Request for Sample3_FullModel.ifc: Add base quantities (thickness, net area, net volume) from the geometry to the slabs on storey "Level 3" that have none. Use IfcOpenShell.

First a look at what the model holds.

```python
import ifcopenshell
import ifcopenshell.util.element
import ifcopenshell.util.unit

model = ifcopenshell.open("Sample3_FullModel.ifc")
print(model.schema)
for unit_type in ("LENGTHUNIT", "AREAUNIT", "VOLUMEUNIT"):
    print(unit_type, ifcopenshell.util.unit.calculate_unit_scale(model, unit_type))
storey = next(s for s in model.by_type("IfcBuildingStorey") if s.Name == "Level 3")
slabs = [e for e in ifcopenshell.util.element.get_decomposition(storey) if e.is_a("IfcSlab")]
for e in sorted(slabs, key=lambda e: e.id()):
    print(e.id(), e.is_a(), e.Name, list(ifcopenshell.util.element.get_psets(e, qtos_only=True)), sep=" | ")
```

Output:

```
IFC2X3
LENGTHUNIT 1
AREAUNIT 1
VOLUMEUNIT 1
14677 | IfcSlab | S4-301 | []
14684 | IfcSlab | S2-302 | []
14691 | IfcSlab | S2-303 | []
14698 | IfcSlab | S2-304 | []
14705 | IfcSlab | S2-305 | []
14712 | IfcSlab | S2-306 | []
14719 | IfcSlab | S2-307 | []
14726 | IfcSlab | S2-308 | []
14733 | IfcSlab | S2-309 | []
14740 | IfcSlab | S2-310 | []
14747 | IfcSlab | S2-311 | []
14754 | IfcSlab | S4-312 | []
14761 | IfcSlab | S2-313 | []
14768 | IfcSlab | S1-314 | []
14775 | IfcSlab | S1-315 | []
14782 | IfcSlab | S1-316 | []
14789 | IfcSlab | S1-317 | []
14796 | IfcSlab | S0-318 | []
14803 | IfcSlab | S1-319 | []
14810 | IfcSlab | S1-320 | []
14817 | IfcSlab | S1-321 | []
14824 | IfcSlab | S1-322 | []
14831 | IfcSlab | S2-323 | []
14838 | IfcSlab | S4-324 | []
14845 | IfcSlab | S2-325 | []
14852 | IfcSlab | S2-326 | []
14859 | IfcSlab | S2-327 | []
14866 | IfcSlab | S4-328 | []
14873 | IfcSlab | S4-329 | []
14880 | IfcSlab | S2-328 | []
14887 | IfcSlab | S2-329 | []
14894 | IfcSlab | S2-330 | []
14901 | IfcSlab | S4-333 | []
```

```python
import ifcopenshell
import ifcopenshell.api.pset
import ifcopenshell.geom
import ifcopenshell.util.element
import ifcopenshell.util.shape
import ifcopenshell.util.unit

model = ifcopenshell.open("Sample3_FullModel.ifc")
unit_scale = ifcopenshell.util.unit.calculate_unit_scale(model)
area_scale = ifcopenshell.util.unit.calculate_unit_scale(model, "AREAUNIT")
volume_scale = ifcopenshell.util.unit.calculate_unit_scale(model, "VOLUMEUNIT")
settings = ifcopenshell.geom.settings()

storey = next(s for s in model.by_type("IfcBuildingStorey") if s.Name == "Level 3")
slabs = [e for e in ifcopenshell.util.element.get_decomposition(storey) if e.is_a("IfcSlab")]

for e in sorted(slabs, key=lambda e: e.id()):
    if ifcopenshell.util.element.get_psets(e, qtos_only=True, should_inherit=False):
        continue
    # Geometry comes back in metres, in the element's own axes.
    shape = ifcopenshell.geom.create_shape(settings, e)
    values = {
        "Width": ifcopenshell.util.shape.get_z(shape.geometry) / unit_scale,
        "NetArea": ifcopenshell.util.shape.get_footprint_area(shape.geometry) / area_scale,
        "NetVolume": ifcopenshell.util.shape.get_volume(shape.geometry) / volume_scale,
    }
    qto = ifcopenshell.api.pset.add_qto(model, product=e, name="BaseQuantities")
    ifcopenshell.api.pset.edit_qto(model, qto=qto, properties=values)
    print(e.id(), {k: round(v, 3) for k, v in values.items()})

model.write("Sample3_FullModel_v2.ifc")
```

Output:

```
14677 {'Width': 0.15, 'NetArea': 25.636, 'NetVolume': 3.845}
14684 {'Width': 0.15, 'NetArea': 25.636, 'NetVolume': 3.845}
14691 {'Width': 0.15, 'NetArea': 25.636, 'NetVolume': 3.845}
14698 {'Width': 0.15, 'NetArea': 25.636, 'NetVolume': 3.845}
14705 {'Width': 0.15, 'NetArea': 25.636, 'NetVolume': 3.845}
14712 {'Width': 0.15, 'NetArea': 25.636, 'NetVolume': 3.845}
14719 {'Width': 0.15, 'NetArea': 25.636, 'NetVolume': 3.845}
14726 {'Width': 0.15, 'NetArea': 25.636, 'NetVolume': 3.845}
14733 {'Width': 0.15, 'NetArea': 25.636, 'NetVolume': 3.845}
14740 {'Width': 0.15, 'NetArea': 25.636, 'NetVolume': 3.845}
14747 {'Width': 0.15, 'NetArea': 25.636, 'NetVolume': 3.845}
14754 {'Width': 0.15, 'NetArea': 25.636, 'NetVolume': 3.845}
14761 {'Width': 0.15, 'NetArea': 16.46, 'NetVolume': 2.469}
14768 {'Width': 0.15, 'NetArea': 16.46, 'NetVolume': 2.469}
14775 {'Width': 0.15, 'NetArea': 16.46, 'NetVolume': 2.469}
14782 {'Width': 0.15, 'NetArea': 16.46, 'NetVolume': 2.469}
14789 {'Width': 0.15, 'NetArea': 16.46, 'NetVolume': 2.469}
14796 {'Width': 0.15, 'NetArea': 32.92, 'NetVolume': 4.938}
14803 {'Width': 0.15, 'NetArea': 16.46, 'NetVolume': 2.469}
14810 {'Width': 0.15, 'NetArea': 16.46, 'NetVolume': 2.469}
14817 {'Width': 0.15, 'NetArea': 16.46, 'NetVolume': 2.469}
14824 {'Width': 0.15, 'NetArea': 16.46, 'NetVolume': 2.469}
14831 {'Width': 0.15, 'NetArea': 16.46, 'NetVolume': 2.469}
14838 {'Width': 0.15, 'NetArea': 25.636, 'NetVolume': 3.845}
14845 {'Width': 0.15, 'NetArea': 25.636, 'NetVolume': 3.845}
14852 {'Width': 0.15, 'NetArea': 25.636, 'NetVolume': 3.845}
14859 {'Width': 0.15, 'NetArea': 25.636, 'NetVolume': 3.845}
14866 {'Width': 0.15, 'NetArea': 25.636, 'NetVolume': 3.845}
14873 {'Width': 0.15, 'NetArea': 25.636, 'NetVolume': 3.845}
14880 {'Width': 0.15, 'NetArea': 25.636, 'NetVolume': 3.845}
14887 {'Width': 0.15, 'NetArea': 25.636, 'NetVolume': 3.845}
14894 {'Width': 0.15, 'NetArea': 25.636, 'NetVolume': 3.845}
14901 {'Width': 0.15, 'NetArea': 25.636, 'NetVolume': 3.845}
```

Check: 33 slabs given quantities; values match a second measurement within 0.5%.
